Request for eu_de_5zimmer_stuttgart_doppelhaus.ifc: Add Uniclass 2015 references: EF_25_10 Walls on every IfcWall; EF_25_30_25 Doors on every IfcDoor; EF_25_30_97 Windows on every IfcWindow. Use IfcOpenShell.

First a look at what the model holds.

```python
import ifcopenshell

model = ifcopenshell.open("eu_de_5zimmer_stuttgart_doppelhaus.ifc")
print(model.schema)
print("classifications:", [c.Name for c in model.by_type("IfcClassification")])
for ifc_class in ("IfcDoor", "IfcRoof", "IfcStair", "IfcWall", "IfcWindow"):
    print(ifc_class, len(model.by_type(ifc_class)))
```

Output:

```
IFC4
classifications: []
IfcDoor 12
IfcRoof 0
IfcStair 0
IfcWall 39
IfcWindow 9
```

```python
import ifcopenshell
import ifcopenshell.api.classification

model = ifcopenshell.open("eu_de_5zimmer_stuttgart_doppelhaus.ifc")

system = ifcopenshell.api.classification.add_classification(model, classification="Uniclass 2015")

codes = {
    "IfcWall": ("EF_25_10", "Walls"),
    "IfcDoor": ("EF_25_30_25", "Doors"),
    "IfcWindow": ("EF_25_30_97", "Windows"),
}
for ifc_class, (code, name) in codes.items():
    products = model.by_type(ifc_class)
    ifcopenshell.api.classification.add_reference(
        model, products=products, classification=system, identification=code, name=name
    )
    print(code, len(products))

model.write("eu_de_5zimmer_stuttgart_doppelhaus_v2.ifc")
```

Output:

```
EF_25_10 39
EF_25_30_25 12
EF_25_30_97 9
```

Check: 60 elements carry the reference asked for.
